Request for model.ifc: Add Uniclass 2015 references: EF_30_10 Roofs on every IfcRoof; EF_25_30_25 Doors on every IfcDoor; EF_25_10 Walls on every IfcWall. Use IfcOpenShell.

First a look at what the model holds.

```python
import ifcopenshell

model = ifcopenshell.open("model.ifc")
print(model.schema)
print("classifications:", [c.Name for c in model.by_type("IfcClassification")])
for ifc_class in ("IfcDoor", "IfcRoof", "IfcStair", "IfcWall", "IfcWindow"):
    print(ifc_class, len(model.by_type(ifc_class)))
```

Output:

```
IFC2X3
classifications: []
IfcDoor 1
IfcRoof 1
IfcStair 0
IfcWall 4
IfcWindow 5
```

```python
import ifcopenshell
import ifcopenshell.api.classification

model = ifcopenshell.open("model.ifc")

# IFC2X3 requires Source and Edition and has no link from the project to the system.
system = model.create_entity("IfcClassification", Source="NBS", Edition="2015", Name="Uniclass 2015")

codes = {
    "IfcRoof": ("EF_30_10", "Roofs"),
    "IfcDoor": ("EF_25_30_25", "Doors"),
    "IfcWall": ("EF_25_10", "Walls"),
}
for ifc_class, (code, name) in codes.items():
    products = model.by_type(ifc_class)
    ifcopenshell.api.classification.add_reference(
        model, products=products, classification=system, identification=code, name=name
    )
    print(code, len(products))

model.write("model_edited.ifc")
```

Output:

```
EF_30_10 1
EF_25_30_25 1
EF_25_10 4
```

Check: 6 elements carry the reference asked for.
